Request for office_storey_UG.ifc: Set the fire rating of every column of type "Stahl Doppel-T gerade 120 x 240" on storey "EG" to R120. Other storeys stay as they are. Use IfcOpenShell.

First a look at what the model holds.

```python
import ifcopenshell
import ifcopenshell.util.element

model = ifcopenshell.open("office_storey_UG.ifc")
print(model.schema)
storey = next(s for s in model.by_type("IfcBuildingStorey") if s.Name == "EG")
columns = [e for e in ifcopenshell.util.element.get_decomposition(storey) if e.is_a("IfcColumn")]
seen = {}
for e in columns:
    element_type = ifcopenshell.util.element.get_type(e)
    key = (element_type.Name if element_type != e and element_type else None, ifcopenshell.util.element.get_pset(e, "Pset_ColumnCommon", "FireRating"))
    seen[key] = seen.get(key, 0) + 1
for (name, value), count in sorted(seen.items(), key=str):
    print(count, "x", name, "|", value)
```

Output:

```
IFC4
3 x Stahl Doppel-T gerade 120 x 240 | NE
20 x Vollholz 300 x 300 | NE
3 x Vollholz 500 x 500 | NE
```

```python
import ifcopenshell
import ifcopenshell.api.pset
import ifcopenshell.util.element

model = ifcopenshell.open("office_storey_UG.ifc")

storey = next(s for s in model.by_type("IfcBuildingStorey") if s.Name == "EG")
columns = [e for e in ifcopenshell.util.element.get_decomposition(storey) if e.is_a("IfcColumn")]

count = 0
for e in columns:
    element_type = ifcopenshell.util.element.get_type(e)
    if element_type in (None, e) or element_type.Name != "Stahl Doppel-T gerade 120 x 240":
        continue
    # add_pset returns the element's existing set when there is one.
    pset = ifcopenshell.api.pset.add_pset(model, product=e, name="Pset_ColumnCommon")
    ifcopenshell.api.pset.edit_pset(model, pset=pset, properties={"FireRating": "R120"})
    count += 1

print(count, "columns updated")

model.write("office_storey_UG-out.ifc")
```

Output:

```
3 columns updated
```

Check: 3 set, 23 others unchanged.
